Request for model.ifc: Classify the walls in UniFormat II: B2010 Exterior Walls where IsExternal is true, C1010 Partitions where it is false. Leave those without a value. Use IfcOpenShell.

First a look at what the model holds.

```python
import ifcopenshell
import ifcopenshell.util.element

model = ifcopenshell.open("model.ifc")
print(model.schema)
print("classifications:", [c.Name for c in model.by_type("IfcClassification")])
values = [ifcopenshell.util.element.get_pset(e, "Pset_WallCommon", "IsExternal") for e in model.by_type("IfcWall")]
for value in (True, False, None):
    print("IsExternal", value, values.count(value))
```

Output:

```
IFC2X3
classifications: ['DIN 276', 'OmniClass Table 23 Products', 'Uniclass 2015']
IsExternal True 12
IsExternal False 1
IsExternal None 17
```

```python
import ifcopenshell
import ifcopenshell.api.classification
import ifcopenshell.util.element

model = ifcopenshell.open("model.ifc")

# IFC2X3 requires Source and Edition and has no link from the project to the system.
system = model.create_entity("IfcClassification", Source="ASTM", Edition="E1557", Name="UniFormat II")

walls = model.by_type("IfcWall")
external = {e: ifcopenshell.util.element.get_pset(e, "Pset_WallCommon", "IsExternal") for e in walls}
for flag, code, name in ((True, "B2010", "Exterior Walls"), (False, "C1010", "Partitions")):
    products = [e for e in walls if external[e] is flag]
    ifcopenshell.api.classification.add_reference(
        model, products=products, classification=system, identification=code, name=name
    )
    print(code, len(products))

model.write("model-out.ifc")
```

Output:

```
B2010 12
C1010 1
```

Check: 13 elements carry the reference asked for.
